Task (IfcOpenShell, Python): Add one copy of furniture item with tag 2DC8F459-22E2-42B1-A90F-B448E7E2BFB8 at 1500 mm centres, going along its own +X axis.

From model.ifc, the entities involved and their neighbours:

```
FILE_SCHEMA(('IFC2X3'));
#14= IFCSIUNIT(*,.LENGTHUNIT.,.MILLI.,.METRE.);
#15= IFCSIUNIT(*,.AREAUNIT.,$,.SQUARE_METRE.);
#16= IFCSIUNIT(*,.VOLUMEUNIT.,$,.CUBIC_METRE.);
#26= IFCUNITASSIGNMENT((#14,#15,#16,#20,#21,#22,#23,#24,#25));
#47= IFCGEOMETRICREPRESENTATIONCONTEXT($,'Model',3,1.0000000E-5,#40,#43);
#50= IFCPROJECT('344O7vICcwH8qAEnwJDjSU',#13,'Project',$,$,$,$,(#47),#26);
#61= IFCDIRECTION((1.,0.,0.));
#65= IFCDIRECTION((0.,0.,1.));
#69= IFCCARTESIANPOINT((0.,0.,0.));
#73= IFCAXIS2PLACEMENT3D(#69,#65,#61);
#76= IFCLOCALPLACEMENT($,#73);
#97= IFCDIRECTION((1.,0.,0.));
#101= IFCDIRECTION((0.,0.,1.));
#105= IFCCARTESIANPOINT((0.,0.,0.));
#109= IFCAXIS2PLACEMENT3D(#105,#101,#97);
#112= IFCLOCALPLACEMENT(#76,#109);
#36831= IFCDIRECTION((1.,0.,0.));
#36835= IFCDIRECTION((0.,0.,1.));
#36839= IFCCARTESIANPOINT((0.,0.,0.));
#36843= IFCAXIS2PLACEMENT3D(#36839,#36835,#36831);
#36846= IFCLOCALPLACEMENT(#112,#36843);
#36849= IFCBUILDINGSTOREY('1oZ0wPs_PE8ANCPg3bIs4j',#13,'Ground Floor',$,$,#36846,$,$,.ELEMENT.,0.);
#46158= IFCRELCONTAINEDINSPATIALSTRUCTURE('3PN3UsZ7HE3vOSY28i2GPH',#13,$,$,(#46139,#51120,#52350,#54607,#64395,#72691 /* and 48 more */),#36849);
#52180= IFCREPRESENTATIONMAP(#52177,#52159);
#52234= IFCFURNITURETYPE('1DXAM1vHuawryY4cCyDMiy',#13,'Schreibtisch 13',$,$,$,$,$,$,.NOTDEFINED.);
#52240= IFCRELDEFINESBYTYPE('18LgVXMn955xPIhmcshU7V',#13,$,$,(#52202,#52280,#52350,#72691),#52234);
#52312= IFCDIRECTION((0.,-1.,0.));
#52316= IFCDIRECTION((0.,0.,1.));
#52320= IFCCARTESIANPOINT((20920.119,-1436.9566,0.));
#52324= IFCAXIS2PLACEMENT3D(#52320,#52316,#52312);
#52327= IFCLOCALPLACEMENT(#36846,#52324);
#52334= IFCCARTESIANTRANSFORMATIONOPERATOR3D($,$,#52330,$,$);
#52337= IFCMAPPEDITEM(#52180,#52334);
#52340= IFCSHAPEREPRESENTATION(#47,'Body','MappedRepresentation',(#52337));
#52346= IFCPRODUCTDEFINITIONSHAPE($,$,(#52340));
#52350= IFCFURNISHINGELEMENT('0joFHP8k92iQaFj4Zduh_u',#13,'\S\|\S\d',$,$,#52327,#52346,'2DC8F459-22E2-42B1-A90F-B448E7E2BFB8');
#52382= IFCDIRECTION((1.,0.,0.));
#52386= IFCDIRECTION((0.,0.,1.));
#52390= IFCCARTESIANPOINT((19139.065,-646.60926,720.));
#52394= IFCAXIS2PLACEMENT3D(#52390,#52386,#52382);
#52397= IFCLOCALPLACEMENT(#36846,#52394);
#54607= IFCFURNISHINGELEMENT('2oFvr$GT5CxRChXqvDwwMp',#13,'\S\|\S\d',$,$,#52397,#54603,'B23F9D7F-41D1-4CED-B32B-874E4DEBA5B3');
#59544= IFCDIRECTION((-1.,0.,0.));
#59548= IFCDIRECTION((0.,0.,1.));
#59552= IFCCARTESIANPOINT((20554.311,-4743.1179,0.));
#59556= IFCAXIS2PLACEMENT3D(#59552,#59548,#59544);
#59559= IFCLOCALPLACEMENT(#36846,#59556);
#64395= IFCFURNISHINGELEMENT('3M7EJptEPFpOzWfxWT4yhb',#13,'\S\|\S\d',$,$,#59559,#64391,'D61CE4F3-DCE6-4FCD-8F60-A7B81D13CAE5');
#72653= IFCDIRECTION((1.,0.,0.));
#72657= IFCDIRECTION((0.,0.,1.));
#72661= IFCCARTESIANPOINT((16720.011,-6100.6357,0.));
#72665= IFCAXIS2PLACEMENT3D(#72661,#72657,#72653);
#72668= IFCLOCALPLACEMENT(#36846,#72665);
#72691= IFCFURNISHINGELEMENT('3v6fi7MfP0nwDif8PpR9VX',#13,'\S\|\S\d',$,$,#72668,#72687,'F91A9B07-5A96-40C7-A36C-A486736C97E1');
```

```python
import ifcopenshell
import ifcopenshell.api.geometry
import ifcopenshell.api.root
import ifcopenshell.util.element
import ifcopenshell.util.placement

model = ifcopenshell.open("model.ifc")


def reuse_history(source, copy):
    """copy_class also copies each property set's owner history, people and application; keep the originals."""
    for rel in copy.IsDefinedBy:
        if rel.is_a("IfcRelDefinesByProperties") and (history := rel.RelatingPropertyDefinition.OwnerHistory):
            rel.RelatingPropertyDefinition.OwnerHistory = source.OwnerHistory
            ifcopenshell.util.element.remove_deep2(model, history)


source = model.by_guid("0joFHP8k92iQaFj4Zduh_u")
base = ifcopenshell.util.placement.get_local_placement(source.ObjectPlacement)
step = base[:3, 0] * 1500.0

for i in range(1, 2):
    copy = ifcopenshell.api.root.copy_class(model, product=source)
    copy.Representation = ifcopenshell.util.element.copy_deep(
        model, source.Representation, exclude=["IfcGeometricRepresentationContext", "IfcRepresentationMap"]
    )
    copy.Tag = None
    reuse_history(source, copy)
    matrix = base.copy()
    matrix[:3, 3] += i * step
    print("added at", matrix[:3, 3].round(3) + 0.0)
    ifcopenshell.api.geometry.edit_object_placement(model, product=copy, matrix=matrix, is_si=False)

model.write("model_rev.ifc")
```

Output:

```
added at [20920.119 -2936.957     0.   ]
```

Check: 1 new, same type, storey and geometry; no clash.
